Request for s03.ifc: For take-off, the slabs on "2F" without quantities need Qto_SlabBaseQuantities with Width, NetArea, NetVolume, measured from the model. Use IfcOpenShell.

First a look at what the model holds.

```python
import ifcopenshell
import ifcopenshell.util.element
import ifcopenshell.util.unit

model = ifcopenshell.open("s03.ifc")
print(model.schema)
for unit_type in ("LENGTHUNIT", "AREAUNIT", "VOLUMEUNIT"):
    print(unit_type, ifcopenshell.util.unit.calculate_unit_scale(model, unit_type))
storey = next(s for s in model.by_type("IfcBuildingStorey") if s.Name == "2F")
slabs = [e for e in ifcopenshell.util.element.get_decomposition(storey) if e.is_a("IfcSlab")]
for e in sorted(slabs, key=lambda e: e.id()):
    print(e.id(), e.is_a(), e.Name, list(ifcopenshell.util.element.get_psets(e, qtos_only=True)), sep=" | ")
```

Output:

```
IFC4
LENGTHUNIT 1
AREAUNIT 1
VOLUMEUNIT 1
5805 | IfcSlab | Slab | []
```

```python
import ifcopenshell
import ifcopenshell.api.pset
import ifcopenshell.geom
import ifcopenshell.util.element
import ifcopenshell.util.shape
import ifcopenshell.util.unit

model = ifcopenshell.open("s03.ifc")
unit_scale = ifcopenshell.util.unit.calculate_unit_scale(model)
area_scale = ifcopenshell.util.unit.calculate_unit_scale(model, "AREAUNIT")
volume_scale = ifcopenshell.util.unit.calculate_unit_scale(model, "VOLUMEUNIT")
settings = ifcopenshell.geom.settings()

storey = next(s for s in model.by_type("IfcBuildingStorey") if s.Name == "2F")
slabs = [e for e in ifcopenshell.util.element.get_decomposition(storey) if e.is_a("IfcSlab")]

for e in sorted(slabs, key=lambda e: e.id()):
    if ifcopenshell.util.element.get_psets(e, qtos_only=True, should_inherit=False):
        continue
    # Geometry comes back in metres, in the element's own axes.
    shape = ifcopenshell.geom.create_shape(settings, e)
    values = {
        "Width": ifcopenshell.util.shape.get_z(shape.geometry) / unit_scale,
        "NetArea": ifcopenshell.util.shape.get_footprint_area(shape.geometry) / area_scale,
        "NetVolume": ifcopenshell.util.shape.get_volume(shape.geometry) / volume_scale,
    }
    qto = ifcopenshell.api.pset.add_qto(model, product=e, name="Qto_SlabBaseQuantities")
    ifcopenshell.api.pset.edit_qto(model, qto=qto, properties=values)
    print(e.id(), {k: round(v, 3) for k, v in values.items()})

model.write("s03_v2.ifc")
```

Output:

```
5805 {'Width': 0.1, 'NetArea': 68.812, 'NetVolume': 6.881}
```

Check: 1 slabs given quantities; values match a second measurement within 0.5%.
